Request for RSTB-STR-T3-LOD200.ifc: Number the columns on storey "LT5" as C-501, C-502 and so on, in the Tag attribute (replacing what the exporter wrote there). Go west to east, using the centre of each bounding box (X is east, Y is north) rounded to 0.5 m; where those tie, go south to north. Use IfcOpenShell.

First a look at what the model holds.

```python
import ifcopenshell
import ifcopenshell.util.element
import ifcopenshell.util.placement

model = ifcopenshell.open("RSTB-STR-T3-LOD200.ifc")
print(model.schema)
storey = next(s for s in model.by_type("IfcBuildingStorey") if s.Name == "LT5")
columns = [e for e in ifcopenshell.util.element.get_decomposition(storey) if e.is_a("IfcColumn")]
for e in sorted(columns, key=lambda e: e.id()):
    origin = ifcopenshell.util.placement.get_local_placement(e.ObjectPlacement)[:3, 3]
    print(e.id(), e.Tag, e.Name, origin.round(2) + 0.0, sep=" | ")
```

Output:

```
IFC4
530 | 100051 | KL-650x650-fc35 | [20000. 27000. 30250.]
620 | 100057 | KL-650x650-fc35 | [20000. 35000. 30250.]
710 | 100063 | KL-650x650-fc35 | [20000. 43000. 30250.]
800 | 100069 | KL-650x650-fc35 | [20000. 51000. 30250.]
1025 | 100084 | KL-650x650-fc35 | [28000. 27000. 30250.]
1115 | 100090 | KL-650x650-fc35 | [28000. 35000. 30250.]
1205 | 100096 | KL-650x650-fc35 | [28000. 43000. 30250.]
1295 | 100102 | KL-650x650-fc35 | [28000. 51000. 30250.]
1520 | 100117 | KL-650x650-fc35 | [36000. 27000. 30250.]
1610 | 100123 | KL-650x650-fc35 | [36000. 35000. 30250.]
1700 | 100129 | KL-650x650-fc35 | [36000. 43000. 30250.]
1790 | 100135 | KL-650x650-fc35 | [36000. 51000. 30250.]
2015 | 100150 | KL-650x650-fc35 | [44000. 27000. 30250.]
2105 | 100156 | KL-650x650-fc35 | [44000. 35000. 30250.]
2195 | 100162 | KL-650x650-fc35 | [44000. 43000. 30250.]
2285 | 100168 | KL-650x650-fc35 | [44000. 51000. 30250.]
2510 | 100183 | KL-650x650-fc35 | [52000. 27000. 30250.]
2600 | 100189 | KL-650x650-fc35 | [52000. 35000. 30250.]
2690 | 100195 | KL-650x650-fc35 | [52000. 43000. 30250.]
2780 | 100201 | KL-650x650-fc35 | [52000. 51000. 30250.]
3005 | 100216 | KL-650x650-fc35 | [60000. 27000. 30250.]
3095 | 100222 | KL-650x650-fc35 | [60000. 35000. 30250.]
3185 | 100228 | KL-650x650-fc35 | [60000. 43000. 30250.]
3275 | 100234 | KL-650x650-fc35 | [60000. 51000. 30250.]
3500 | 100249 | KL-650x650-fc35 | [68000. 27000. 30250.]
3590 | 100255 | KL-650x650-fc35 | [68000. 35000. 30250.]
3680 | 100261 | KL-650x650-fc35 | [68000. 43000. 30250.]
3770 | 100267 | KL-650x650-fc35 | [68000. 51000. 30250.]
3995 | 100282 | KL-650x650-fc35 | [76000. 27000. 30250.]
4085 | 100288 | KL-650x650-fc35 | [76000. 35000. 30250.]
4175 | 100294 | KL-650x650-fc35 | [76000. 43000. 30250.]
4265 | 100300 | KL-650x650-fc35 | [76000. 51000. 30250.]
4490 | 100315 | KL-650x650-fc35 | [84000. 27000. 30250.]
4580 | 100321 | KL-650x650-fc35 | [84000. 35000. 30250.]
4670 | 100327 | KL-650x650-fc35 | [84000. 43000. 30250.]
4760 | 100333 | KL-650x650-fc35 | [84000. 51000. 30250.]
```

```python
import ifcopenshell
import ifcopenshell.geom
import ifcopenshell.util.element
import ifcopenshell.util.shape

model = ifcopenshell.open("RSTB-STR-T3-LOD200.ifc")
settings = ifcopenshell.geom.settings()
settings.set("use-world-coords", True)


def centre(element):
    shape = ifcopenshell.geom.create_shape(settings, element)
    return ifcopenshell.util.shape.get_bbox_centroid(shape.geometry)


storey = next(s for s in model.by_type("IfcBuildingStorey") if s.Name == "LT5")
columns = [e for e in ifcopenshell.util.element.get_decomposition(storey) if e.is_a("IfcColumn")]

# Insertion points can sit at a corner or the storey origin, so sort by the geometry (in metres).
centres = {e: centre(e) for e in columns}
columns.sort(key=lambda e: (round(centres[e][0] / 0.5), centres[e][1]))

for i, e in enumerate(columns, start=1):
    number = f"C-5{i:02d}"
    e.Tag = number
    print(e.id(), number)

model.write("RSTB-STR-T3-LOD200_rev.ifc")
```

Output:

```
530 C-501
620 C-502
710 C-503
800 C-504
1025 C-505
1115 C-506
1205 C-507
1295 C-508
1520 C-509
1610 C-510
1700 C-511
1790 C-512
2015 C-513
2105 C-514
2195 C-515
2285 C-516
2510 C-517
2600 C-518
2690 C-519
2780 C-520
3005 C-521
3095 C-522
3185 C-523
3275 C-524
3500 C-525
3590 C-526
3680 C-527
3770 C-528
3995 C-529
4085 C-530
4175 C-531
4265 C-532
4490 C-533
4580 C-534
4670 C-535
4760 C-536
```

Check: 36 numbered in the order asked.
